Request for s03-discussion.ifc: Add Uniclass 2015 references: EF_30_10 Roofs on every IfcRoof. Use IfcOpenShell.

First a look at what the model holds.

```python
import ifcopenshell

model = ifcopenshell.open("s03-discussion.ifc")
print(model.schema)
print("classifications:", [c.Name for c in model.by_type("IfcClassification")])
for ifc_class in ("IfcDoor", "IfcRoof", "IfcStair", "IfcWall", "IfcWindow"):
    print(ifc_class, len(model.by_type(ifc_class)))
```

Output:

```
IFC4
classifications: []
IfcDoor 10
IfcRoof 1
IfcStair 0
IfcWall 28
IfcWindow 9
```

```python
import ifcopenshell
import ifcopenshell.api.classification

model = ifcopenshell.open("s03-discussion.ifc")

system = ifcopenshell.api.classification.add_classification(model, classification="Uniclass 2015")

codes = {
    "IfcRoof": ("EF_30_10", "Roofs"),
}
for ifc_class, (code, name) in codes.items():
    products = model.by_type(ifc_class)
    ifcopenshell.api.classification.add_reference(
        model, products=products, classification=system, identification=code, name=name
    )
    print(code, len(products))

model.write("s03-discussion_updated.ifc")
```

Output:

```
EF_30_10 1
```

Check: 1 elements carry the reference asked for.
